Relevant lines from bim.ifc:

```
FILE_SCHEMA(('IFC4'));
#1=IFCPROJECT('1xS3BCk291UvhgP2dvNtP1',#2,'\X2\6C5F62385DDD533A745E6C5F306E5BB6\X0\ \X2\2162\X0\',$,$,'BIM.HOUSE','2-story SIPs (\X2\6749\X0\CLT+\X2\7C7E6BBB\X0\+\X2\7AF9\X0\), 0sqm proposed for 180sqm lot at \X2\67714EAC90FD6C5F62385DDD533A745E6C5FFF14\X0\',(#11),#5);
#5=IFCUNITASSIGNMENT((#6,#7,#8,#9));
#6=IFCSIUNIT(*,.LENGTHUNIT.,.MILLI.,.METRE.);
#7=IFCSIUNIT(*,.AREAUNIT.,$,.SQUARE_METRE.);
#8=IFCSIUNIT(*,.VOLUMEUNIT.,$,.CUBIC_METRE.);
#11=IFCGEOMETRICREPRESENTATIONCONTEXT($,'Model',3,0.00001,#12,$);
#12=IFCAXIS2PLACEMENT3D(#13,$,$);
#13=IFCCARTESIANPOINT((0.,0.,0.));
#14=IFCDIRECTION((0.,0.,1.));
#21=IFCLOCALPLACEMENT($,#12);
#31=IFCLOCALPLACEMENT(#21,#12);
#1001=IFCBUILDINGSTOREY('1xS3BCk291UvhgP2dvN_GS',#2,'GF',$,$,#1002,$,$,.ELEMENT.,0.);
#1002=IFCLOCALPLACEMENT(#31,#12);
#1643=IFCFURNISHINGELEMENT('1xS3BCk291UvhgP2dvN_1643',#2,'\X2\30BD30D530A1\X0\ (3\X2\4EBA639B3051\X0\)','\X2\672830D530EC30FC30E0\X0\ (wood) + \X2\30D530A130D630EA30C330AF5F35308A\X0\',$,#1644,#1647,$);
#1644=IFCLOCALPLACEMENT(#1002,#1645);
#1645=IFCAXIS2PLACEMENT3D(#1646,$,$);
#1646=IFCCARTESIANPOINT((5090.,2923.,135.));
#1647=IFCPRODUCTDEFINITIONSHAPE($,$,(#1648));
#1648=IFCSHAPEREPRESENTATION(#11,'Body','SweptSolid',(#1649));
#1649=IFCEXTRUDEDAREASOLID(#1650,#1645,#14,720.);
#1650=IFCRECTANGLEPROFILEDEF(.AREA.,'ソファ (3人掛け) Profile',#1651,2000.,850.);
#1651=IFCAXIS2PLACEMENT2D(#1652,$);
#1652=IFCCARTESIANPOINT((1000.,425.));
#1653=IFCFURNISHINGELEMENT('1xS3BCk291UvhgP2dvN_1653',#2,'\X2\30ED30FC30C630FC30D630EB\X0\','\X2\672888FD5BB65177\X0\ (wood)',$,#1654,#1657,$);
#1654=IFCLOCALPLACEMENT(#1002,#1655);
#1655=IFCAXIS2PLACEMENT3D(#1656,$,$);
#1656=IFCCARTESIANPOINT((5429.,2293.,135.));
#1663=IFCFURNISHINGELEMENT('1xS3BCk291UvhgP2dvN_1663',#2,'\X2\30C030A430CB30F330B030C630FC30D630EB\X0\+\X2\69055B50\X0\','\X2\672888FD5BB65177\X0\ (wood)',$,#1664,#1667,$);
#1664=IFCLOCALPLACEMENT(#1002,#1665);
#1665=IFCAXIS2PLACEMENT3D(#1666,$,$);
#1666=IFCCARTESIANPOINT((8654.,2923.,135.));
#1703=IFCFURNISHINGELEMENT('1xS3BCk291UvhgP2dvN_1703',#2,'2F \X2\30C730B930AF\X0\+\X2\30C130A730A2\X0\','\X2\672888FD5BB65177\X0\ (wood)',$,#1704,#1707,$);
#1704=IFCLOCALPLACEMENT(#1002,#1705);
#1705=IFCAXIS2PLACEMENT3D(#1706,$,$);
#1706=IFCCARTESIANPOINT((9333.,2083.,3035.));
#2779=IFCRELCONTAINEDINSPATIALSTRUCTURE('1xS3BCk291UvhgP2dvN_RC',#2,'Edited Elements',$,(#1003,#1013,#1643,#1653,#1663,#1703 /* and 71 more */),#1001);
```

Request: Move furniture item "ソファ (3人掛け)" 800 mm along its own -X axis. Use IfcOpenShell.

```python
import ifcopenshell
import ifcopenshell.api.geometry
import ifcopenshell.util.placement

model = ifcopenshell.open("bim.ifc")

item = model.by_id(1643)
matrix = ifcopenshell.util.placement.get_local_placement(item.ObjectPlacement)
matrix[:3, 3] -= matrix[:3, 0] * 800.0
ifcopenshell.api.geometry.edit_object_placement(model, product=item, matrix=matrix, is_si=False)

print(ifcopenshell.util.placement.get_local_placement(item.ObjectPlacement).round(3) + 0.0)

model.write("bim_rev.ifc")
```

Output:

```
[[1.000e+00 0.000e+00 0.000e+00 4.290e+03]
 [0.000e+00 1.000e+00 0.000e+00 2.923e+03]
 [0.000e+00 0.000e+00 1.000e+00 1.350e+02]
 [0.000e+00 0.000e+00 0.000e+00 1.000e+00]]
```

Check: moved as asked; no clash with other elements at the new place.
